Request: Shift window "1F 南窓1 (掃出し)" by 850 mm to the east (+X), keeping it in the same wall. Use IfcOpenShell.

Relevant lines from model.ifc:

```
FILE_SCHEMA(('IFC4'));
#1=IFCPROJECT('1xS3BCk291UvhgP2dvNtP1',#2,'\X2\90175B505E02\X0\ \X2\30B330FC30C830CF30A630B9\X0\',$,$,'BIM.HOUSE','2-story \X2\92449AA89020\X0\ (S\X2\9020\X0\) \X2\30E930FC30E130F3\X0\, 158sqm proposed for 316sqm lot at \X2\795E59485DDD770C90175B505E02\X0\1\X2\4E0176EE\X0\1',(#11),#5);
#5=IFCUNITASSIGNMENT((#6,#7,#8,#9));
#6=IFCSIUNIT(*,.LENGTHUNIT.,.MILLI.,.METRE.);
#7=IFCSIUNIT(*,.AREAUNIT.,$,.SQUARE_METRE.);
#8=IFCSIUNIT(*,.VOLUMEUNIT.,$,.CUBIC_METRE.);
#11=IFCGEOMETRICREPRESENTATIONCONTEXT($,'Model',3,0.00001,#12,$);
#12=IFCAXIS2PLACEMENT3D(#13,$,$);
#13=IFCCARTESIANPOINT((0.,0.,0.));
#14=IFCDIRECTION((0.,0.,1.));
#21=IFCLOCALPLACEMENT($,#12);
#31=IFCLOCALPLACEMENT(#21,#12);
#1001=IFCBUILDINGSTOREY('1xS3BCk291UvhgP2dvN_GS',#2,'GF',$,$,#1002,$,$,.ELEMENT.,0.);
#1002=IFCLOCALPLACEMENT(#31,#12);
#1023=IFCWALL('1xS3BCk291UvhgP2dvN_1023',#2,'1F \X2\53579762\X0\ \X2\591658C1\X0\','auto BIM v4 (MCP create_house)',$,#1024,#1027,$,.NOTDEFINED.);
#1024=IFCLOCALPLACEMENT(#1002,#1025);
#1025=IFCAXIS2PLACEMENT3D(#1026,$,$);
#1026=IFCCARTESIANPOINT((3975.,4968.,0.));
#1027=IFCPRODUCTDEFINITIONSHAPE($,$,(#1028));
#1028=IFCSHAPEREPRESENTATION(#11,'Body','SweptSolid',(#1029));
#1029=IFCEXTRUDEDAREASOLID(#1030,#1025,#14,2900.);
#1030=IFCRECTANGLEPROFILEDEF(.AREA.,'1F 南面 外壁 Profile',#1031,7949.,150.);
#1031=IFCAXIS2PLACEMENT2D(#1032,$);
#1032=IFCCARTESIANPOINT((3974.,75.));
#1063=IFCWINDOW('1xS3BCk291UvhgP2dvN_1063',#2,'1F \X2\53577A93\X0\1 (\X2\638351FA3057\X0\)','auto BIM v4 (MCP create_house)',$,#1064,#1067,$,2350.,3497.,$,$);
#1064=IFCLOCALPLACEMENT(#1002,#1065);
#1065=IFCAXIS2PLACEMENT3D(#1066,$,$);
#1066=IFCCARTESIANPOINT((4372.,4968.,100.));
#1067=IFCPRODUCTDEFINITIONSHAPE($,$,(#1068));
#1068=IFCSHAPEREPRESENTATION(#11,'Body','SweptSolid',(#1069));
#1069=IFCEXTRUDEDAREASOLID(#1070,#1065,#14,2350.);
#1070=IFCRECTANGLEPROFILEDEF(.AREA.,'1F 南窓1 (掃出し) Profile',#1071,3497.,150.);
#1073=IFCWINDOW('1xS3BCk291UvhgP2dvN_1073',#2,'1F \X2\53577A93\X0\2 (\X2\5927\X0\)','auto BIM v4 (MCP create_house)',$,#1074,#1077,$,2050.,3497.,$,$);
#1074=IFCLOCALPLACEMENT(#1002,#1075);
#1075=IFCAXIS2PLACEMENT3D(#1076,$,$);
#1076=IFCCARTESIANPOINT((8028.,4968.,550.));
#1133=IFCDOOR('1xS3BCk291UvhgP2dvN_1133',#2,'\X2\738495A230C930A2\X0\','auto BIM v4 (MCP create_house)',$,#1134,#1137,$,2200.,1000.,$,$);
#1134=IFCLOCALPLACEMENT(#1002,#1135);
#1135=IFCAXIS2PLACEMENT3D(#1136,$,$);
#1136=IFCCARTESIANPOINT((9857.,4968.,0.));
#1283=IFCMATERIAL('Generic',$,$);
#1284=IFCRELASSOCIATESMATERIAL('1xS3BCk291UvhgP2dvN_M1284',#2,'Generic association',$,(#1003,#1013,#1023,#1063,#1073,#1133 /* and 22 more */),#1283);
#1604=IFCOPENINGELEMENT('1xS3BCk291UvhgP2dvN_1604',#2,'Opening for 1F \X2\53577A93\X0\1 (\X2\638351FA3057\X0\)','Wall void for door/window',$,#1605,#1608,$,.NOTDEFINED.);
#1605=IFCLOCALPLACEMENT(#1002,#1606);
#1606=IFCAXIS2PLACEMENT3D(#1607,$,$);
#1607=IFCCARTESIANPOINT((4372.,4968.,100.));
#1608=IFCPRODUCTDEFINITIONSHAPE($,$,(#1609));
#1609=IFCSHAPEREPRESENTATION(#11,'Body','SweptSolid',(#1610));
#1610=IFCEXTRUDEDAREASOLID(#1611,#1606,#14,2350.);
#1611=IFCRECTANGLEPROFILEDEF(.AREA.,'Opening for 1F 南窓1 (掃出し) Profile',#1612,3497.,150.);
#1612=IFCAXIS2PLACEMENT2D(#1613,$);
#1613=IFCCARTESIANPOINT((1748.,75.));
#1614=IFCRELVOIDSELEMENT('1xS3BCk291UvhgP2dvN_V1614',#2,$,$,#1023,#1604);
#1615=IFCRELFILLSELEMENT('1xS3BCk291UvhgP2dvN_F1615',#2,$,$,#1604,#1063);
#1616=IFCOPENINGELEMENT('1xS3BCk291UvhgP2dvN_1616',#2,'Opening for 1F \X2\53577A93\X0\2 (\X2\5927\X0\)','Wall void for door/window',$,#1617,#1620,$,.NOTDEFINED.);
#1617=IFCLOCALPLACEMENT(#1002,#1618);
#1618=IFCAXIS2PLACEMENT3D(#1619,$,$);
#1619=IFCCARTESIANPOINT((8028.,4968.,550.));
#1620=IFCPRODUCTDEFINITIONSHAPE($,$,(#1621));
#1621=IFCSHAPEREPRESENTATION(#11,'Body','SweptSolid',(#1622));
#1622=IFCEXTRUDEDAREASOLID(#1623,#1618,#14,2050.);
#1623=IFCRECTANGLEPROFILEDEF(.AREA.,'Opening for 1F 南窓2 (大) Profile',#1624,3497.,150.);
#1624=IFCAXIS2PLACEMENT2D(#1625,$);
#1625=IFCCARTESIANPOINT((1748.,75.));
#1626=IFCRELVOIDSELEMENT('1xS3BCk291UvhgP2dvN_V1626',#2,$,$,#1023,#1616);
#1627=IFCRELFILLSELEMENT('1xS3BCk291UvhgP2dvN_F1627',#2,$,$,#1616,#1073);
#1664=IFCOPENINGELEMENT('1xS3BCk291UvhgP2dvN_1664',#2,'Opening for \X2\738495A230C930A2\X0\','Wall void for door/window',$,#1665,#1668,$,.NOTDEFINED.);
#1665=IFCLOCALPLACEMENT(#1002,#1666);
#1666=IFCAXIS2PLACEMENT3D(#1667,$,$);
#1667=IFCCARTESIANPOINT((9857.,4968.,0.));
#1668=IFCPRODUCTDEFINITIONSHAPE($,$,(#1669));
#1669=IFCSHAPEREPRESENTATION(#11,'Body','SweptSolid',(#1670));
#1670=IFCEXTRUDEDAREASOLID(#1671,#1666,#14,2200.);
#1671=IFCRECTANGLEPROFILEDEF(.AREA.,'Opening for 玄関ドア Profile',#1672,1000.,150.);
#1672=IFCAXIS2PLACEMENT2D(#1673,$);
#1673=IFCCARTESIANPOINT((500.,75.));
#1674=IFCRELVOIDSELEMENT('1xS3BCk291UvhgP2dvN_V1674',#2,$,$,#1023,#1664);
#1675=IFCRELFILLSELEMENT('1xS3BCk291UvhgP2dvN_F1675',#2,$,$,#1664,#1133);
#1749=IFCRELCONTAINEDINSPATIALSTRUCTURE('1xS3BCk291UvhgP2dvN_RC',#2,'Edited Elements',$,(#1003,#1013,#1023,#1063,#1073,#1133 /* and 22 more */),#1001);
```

```python
import ifcopenshell
import ifcopenshell.api.geometry
import ifcopenshell.util.placement

model = ifcopenshell.open("model.ifc")

window = model.by_guid("1xS3BCk291UvhgP2dvN_1063")
opening = window.FillsVoids[0].RelatingOpeningElement
wall = opening.VoidsElements[0].RelatingBuildingElement

wall_matrix = ifcopenshell.util.placement.get_local_placement(wall.ObjectPlacement)
shift = wall_matrix[:3, 0] * 850.0
before = ifcopenshell.util.placement.get_local_placement(window.ObjectPlacement)[:3, 3].copy()

# The window is not placed relative to its opening, so move both.
for product in (opening, window):
    matrix = ifcopenshell.util.placement.get_local_placement(product.ObjectPlacement)
    matrix[:3, 3] += shift
    ifcopenshell.api.geometry.edit_object_placement(model, product=product, matrix=matrix, is_si=False)

after = ifcopenshell.util.placement.get_local_placement(window.ObjectPlacement)[:3, 3]
print("window moved by", (after - before).round(3) + 0.0)

model.write("model-out.ifc")
```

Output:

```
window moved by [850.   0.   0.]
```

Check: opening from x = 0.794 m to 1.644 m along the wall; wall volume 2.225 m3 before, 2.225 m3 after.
